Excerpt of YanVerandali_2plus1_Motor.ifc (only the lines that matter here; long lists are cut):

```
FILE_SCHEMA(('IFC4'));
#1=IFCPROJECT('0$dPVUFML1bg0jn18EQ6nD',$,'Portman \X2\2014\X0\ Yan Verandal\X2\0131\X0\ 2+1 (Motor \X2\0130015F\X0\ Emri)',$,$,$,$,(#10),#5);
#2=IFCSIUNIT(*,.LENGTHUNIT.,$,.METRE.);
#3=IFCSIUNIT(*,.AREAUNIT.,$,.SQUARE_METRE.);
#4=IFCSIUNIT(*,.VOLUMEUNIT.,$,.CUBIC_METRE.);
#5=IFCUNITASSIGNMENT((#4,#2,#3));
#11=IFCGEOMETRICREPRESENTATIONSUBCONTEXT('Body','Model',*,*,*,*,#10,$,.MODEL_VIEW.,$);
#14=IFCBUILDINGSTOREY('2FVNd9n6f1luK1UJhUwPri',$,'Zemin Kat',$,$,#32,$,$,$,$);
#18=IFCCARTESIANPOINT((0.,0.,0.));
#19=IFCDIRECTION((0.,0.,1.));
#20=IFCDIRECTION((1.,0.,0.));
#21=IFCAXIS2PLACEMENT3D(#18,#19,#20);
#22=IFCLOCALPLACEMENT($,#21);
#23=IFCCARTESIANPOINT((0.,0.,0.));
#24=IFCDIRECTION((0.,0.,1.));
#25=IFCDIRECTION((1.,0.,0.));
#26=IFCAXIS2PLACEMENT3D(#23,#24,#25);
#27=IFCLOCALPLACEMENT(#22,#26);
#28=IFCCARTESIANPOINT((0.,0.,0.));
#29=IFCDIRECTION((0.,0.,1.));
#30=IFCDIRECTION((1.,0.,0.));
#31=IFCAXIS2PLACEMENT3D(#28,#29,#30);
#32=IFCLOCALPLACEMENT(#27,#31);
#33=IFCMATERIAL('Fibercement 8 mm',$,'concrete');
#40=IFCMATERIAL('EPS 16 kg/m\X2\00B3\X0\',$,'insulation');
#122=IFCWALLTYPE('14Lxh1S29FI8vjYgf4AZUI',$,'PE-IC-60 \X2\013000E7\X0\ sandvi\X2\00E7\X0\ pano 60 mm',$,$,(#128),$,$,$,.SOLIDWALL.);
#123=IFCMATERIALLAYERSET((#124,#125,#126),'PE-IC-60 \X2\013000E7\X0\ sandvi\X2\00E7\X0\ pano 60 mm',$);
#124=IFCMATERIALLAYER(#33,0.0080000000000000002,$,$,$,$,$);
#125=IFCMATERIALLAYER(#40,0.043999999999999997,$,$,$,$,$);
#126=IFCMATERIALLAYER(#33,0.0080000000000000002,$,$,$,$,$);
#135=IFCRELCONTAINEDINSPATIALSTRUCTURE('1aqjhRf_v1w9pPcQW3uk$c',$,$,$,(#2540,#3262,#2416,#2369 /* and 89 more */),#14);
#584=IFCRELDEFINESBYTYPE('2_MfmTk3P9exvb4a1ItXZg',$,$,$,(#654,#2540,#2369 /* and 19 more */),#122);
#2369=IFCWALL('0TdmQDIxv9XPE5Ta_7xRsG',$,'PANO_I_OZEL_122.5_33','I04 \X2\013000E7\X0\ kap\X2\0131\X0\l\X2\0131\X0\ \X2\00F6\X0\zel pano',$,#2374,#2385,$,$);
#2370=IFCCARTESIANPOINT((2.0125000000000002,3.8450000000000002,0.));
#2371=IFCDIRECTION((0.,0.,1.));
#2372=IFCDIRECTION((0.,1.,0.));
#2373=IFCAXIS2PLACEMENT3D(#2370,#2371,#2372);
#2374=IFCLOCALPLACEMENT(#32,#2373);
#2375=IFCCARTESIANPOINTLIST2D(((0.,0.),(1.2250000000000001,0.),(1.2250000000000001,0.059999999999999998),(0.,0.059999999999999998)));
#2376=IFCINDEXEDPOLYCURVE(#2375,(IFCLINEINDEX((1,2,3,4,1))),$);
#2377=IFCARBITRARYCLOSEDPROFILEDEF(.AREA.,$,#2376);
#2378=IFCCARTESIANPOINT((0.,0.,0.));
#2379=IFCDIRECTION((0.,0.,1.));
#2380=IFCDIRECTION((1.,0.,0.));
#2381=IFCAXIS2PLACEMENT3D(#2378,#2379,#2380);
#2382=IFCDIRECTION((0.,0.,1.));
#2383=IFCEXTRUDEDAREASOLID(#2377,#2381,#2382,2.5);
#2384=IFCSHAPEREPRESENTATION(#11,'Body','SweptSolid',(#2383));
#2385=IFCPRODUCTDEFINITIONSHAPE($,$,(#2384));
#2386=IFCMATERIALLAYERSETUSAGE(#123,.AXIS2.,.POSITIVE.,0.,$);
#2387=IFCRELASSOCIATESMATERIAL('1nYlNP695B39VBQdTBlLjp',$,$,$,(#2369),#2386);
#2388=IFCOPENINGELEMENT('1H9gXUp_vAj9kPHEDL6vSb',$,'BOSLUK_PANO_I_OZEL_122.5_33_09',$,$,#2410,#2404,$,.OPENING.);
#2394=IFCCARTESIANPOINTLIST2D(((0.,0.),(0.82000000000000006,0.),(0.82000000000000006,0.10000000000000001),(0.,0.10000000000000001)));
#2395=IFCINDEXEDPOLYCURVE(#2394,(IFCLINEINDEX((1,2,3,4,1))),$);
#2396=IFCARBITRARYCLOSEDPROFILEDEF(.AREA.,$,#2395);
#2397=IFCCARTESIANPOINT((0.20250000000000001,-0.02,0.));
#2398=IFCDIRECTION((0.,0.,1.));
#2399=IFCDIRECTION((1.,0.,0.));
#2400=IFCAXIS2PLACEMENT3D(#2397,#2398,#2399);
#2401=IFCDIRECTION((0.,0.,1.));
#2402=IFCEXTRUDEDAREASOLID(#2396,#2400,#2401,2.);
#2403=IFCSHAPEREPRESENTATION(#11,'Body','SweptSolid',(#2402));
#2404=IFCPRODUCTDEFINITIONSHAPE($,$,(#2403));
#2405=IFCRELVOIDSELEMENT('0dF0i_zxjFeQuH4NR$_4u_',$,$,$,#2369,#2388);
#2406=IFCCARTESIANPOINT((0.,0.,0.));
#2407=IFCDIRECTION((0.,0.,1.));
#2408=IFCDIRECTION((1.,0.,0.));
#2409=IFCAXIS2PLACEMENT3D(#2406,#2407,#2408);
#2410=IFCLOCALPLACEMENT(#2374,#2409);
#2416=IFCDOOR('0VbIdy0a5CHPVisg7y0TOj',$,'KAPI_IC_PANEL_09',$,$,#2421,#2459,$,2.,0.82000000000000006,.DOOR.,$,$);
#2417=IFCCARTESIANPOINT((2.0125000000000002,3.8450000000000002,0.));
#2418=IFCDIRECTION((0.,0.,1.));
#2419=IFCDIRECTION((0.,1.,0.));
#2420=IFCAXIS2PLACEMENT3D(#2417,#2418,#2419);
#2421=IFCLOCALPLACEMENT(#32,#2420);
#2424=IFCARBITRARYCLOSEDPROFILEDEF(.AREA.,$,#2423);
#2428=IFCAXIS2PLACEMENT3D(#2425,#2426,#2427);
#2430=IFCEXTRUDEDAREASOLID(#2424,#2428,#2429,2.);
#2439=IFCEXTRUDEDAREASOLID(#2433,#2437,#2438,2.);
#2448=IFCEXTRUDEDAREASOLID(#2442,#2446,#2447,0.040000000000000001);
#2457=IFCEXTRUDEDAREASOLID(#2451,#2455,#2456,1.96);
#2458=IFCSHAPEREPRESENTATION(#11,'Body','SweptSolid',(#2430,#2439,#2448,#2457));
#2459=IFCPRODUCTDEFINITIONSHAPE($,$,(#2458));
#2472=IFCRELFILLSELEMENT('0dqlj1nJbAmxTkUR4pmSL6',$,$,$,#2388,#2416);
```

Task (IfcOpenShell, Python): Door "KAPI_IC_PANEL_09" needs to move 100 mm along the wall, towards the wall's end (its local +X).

```python
import ifcopenshell
import ifcopenshell.api.geometry
import ifcopenshell.util.placement
import ifcopenshell.util.unit

model = ifcopenshell.open("YanVerandali_2plus1_Motor.ifc")
unit_scale = ifcopenshell.util.unit.calculate_unit_scale(model)

door = model.by_guid("0VbIdy0a5CHPVisg7y0TOj")
opening = door.FillsVoids[0].RelatingOpeningElement
wall = opening.VoidsElements[0].RelatingBuildingElement

wall_matrix = ifcopenshell.util.placement.get_local_placement(wall.ObjectPlacement)
shift = wall_matrix[:3, 0] * 0.1 / unit_scale
before = ifcopenshell.util.placement.get_local_placement(door.ObjectPlacement)[:3, 3].copy()

# The door is not placed relative to its opening, so move both.
for product in (opening, door):
    matrix = ifcopenshell.util.placement.get_local_placement(product.ObjectPlacement)
    matrix[:3, 3] += shift
    ifcopenshell.api.geometry.edit_object_placement(model, product=product, matrix=matrix, is_si=False)

after = ifcopenshell.util.placement.get_local_placement(door.ObjectPlacement)[:3, 3]
print("door moved by", (after - before).round(3) + 0.0)

model.write("YanVerandali_2plus1_Motor_edited.ifc")
```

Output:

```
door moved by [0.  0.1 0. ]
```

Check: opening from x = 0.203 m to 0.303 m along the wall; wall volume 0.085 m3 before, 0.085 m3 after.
